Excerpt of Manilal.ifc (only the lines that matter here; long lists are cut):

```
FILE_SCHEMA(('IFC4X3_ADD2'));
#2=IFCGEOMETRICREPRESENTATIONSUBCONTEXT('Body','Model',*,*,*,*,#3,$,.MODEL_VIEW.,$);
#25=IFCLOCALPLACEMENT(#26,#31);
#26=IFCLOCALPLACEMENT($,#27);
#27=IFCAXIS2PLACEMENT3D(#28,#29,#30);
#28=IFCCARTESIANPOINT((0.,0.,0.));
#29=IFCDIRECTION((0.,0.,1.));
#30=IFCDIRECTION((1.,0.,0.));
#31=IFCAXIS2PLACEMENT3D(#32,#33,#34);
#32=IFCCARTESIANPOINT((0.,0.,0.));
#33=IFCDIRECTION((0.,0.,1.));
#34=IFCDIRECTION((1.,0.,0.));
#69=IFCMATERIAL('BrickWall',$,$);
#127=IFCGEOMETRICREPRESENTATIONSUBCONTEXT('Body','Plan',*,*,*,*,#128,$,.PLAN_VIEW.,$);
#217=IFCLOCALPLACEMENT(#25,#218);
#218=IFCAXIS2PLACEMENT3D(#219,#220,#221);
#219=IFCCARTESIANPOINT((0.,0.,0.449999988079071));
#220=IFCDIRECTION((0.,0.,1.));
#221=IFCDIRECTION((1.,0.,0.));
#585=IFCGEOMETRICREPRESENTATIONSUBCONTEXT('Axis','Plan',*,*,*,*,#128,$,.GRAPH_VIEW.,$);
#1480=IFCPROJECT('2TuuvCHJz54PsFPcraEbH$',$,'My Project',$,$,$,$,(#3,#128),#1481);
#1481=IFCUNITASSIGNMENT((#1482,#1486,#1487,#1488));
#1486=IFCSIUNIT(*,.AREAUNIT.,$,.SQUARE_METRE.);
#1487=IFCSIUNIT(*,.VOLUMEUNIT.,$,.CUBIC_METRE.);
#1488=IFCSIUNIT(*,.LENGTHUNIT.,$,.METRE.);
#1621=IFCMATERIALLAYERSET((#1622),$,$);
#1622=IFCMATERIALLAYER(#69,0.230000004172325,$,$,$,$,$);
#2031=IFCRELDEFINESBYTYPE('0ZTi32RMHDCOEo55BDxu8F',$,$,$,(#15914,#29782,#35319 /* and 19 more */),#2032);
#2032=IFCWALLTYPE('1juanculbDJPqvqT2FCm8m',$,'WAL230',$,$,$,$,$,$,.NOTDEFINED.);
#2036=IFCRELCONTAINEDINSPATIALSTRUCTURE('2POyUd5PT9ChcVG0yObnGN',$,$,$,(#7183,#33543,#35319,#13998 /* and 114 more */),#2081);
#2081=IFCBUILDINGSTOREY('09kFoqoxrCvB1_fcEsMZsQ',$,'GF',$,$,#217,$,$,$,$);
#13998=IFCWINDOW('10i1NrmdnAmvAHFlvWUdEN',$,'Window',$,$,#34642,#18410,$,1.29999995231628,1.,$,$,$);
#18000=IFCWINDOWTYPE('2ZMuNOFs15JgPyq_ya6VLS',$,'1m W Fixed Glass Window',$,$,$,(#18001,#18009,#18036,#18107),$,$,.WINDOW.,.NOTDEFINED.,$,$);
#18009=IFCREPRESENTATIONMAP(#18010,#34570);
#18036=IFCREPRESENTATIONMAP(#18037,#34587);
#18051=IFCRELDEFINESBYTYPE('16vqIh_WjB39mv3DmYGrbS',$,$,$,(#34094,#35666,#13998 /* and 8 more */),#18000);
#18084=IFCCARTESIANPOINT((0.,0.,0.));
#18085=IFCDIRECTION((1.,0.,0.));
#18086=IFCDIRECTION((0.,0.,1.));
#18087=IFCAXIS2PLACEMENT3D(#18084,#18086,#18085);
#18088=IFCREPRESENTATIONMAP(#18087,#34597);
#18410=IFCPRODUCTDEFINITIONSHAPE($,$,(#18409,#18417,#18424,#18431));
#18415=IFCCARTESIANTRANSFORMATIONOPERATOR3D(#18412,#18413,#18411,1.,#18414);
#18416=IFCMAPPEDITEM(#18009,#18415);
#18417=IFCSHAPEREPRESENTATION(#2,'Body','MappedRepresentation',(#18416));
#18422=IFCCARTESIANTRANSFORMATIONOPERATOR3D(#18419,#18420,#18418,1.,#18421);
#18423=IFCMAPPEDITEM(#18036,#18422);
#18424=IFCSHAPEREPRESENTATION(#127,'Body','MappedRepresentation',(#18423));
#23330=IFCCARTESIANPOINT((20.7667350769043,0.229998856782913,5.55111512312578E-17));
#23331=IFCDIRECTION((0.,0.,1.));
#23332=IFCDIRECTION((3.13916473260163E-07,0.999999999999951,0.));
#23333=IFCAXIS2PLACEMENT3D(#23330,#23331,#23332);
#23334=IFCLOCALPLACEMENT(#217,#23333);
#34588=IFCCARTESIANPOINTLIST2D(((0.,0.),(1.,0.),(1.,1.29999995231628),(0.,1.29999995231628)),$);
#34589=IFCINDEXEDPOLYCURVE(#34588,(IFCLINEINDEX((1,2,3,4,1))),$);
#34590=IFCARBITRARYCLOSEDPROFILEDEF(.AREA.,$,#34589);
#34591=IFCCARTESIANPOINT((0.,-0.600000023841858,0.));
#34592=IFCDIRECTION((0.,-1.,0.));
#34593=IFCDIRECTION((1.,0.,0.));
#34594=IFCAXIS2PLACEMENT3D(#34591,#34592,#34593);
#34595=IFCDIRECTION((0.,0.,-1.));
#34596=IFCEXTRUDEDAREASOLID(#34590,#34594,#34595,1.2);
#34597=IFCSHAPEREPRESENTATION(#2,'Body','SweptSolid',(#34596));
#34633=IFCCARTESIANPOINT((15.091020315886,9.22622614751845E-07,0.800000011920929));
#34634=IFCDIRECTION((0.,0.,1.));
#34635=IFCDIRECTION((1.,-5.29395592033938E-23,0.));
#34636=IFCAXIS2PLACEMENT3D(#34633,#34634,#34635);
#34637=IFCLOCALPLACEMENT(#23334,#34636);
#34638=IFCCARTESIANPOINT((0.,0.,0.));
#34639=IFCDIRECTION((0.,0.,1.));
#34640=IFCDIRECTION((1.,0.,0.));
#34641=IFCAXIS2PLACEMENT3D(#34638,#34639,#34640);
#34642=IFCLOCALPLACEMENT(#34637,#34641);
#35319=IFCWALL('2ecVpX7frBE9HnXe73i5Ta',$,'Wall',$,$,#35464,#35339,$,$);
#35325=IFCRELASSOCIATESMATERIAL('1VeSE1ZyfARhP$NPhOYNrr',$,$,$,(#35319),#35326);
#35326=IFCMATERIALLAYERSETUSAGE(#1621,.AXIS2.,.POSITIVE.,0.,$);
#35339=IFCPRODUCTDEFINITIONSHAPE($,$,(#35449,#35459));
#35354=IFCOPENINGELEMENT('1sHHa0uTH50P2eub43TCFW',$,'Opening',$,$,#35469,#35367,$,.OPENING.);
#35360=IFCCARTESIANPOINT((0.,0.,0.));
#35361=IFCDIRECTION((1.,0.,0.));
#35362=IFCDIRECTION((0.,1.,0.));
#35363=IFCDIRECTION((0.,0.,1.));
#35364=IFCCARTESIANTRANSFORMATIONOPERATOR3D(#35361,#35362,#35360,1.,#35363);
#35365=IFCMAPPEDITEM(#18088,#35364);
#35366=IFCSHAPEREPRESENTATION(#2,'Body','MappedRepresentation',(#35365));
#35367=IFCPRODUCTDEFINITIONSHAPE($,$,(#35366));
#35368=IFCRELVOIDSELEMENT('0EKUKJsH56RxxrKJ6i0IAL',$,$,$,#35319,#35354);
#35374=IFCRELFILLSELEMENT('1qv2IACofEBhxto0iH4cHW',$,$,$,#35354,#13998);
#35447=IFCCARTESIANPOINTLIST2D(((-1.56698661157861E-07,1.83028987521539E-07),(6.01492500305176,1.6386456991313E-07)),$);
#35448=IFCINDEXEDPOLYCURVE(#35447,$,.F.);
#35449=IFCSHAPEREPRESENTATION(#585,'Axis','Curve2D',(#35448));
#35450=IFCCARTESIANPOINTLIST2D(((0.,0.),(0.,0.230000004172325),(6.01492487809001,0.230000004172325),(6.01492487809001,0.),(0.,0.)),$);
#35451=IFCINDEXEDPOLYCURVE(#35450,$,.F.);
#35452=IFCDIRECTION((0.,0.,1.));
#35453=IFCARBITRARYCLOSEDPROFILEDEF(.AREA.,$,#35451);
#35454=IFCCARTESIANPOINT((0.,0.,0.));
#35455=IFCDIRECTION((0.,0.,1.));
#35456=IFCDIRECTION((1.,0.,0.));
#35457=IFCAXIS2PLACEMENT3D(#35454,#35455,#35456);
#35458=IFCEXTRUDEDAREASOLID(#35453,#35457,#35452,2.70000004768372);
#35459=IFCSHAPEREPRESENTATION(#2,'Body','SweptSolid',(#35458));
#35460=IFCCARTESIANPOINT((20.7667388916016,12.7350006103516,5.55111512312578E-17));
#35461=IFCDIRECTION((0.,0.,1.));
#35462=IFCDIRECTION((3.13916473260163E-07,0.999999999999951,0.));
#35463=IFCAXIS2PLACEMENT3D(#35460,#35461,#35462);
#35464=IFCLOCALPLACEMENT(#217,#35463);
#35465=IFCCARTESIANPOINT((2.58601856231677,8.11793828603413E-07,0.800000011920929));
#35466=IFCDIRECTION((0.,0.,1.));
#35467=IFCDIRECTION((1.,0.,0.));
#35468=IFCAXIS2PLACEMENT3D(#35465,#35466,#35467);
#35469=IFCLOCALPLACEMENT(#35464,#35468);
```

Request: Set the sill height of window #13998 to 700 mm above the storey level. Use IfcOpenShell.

```python
import numpy as np
import ifcopenshell
import ifcopenshell.api.geometry
import ifcopenshell.geom
import ifcopenshell.util.element
import ifcopenshell.util.placement
import ifcopenshell.util.shape
import ifcopenshell.util.unit

model = ifcopenshell.open("Manilal.ifc")
unit_scale = ifcopenshell.util.unit.calculate_unit_scale(model)

window = model.by_guid("10i1NrmdnAmvAHFlvWUdEN")
opening = window.FillsVoids[0].RelatingOpeningElement
storey = ifcopenshell.util.element.get_container(window, ifc_class="IfcBuildingStorey")
level = ifcopenshell.util.placement.get_local_placement(storey.ObjectPlacement)[2, 3]

# The opening's origin need not be at the sill, so measure its lowest point.
shape = ifcopenshell.geom.create_shape(ifcopenshell.geom.settings(), opening)
bottom = ifcopenshell.util.shape.get_shape_bottom_elevation(shape, shape.geometry) / unit_scale
dz = level + 0.7 / unit_scale - bottom

shift = np.array([0.0, 0.0, dz])
# The window is not placed relative to its opening, so move both.
for product in (opening, window):
    matrix = ifcopenshell.util.placement.get_local_placement(product.ObjectPlacement)
    matrix[:3, 3] += shift
    ifcopenshell.api.geometry.edit_object_placement(model, product=product, matrix=matrix, is_si=False)

print(f"moved by {dz * unit_scale:+.3f} m")

model.write("Manilal_v2.ifc")
```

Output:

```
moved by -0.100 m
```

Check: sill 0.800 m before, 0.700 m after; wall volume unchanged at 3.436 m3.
